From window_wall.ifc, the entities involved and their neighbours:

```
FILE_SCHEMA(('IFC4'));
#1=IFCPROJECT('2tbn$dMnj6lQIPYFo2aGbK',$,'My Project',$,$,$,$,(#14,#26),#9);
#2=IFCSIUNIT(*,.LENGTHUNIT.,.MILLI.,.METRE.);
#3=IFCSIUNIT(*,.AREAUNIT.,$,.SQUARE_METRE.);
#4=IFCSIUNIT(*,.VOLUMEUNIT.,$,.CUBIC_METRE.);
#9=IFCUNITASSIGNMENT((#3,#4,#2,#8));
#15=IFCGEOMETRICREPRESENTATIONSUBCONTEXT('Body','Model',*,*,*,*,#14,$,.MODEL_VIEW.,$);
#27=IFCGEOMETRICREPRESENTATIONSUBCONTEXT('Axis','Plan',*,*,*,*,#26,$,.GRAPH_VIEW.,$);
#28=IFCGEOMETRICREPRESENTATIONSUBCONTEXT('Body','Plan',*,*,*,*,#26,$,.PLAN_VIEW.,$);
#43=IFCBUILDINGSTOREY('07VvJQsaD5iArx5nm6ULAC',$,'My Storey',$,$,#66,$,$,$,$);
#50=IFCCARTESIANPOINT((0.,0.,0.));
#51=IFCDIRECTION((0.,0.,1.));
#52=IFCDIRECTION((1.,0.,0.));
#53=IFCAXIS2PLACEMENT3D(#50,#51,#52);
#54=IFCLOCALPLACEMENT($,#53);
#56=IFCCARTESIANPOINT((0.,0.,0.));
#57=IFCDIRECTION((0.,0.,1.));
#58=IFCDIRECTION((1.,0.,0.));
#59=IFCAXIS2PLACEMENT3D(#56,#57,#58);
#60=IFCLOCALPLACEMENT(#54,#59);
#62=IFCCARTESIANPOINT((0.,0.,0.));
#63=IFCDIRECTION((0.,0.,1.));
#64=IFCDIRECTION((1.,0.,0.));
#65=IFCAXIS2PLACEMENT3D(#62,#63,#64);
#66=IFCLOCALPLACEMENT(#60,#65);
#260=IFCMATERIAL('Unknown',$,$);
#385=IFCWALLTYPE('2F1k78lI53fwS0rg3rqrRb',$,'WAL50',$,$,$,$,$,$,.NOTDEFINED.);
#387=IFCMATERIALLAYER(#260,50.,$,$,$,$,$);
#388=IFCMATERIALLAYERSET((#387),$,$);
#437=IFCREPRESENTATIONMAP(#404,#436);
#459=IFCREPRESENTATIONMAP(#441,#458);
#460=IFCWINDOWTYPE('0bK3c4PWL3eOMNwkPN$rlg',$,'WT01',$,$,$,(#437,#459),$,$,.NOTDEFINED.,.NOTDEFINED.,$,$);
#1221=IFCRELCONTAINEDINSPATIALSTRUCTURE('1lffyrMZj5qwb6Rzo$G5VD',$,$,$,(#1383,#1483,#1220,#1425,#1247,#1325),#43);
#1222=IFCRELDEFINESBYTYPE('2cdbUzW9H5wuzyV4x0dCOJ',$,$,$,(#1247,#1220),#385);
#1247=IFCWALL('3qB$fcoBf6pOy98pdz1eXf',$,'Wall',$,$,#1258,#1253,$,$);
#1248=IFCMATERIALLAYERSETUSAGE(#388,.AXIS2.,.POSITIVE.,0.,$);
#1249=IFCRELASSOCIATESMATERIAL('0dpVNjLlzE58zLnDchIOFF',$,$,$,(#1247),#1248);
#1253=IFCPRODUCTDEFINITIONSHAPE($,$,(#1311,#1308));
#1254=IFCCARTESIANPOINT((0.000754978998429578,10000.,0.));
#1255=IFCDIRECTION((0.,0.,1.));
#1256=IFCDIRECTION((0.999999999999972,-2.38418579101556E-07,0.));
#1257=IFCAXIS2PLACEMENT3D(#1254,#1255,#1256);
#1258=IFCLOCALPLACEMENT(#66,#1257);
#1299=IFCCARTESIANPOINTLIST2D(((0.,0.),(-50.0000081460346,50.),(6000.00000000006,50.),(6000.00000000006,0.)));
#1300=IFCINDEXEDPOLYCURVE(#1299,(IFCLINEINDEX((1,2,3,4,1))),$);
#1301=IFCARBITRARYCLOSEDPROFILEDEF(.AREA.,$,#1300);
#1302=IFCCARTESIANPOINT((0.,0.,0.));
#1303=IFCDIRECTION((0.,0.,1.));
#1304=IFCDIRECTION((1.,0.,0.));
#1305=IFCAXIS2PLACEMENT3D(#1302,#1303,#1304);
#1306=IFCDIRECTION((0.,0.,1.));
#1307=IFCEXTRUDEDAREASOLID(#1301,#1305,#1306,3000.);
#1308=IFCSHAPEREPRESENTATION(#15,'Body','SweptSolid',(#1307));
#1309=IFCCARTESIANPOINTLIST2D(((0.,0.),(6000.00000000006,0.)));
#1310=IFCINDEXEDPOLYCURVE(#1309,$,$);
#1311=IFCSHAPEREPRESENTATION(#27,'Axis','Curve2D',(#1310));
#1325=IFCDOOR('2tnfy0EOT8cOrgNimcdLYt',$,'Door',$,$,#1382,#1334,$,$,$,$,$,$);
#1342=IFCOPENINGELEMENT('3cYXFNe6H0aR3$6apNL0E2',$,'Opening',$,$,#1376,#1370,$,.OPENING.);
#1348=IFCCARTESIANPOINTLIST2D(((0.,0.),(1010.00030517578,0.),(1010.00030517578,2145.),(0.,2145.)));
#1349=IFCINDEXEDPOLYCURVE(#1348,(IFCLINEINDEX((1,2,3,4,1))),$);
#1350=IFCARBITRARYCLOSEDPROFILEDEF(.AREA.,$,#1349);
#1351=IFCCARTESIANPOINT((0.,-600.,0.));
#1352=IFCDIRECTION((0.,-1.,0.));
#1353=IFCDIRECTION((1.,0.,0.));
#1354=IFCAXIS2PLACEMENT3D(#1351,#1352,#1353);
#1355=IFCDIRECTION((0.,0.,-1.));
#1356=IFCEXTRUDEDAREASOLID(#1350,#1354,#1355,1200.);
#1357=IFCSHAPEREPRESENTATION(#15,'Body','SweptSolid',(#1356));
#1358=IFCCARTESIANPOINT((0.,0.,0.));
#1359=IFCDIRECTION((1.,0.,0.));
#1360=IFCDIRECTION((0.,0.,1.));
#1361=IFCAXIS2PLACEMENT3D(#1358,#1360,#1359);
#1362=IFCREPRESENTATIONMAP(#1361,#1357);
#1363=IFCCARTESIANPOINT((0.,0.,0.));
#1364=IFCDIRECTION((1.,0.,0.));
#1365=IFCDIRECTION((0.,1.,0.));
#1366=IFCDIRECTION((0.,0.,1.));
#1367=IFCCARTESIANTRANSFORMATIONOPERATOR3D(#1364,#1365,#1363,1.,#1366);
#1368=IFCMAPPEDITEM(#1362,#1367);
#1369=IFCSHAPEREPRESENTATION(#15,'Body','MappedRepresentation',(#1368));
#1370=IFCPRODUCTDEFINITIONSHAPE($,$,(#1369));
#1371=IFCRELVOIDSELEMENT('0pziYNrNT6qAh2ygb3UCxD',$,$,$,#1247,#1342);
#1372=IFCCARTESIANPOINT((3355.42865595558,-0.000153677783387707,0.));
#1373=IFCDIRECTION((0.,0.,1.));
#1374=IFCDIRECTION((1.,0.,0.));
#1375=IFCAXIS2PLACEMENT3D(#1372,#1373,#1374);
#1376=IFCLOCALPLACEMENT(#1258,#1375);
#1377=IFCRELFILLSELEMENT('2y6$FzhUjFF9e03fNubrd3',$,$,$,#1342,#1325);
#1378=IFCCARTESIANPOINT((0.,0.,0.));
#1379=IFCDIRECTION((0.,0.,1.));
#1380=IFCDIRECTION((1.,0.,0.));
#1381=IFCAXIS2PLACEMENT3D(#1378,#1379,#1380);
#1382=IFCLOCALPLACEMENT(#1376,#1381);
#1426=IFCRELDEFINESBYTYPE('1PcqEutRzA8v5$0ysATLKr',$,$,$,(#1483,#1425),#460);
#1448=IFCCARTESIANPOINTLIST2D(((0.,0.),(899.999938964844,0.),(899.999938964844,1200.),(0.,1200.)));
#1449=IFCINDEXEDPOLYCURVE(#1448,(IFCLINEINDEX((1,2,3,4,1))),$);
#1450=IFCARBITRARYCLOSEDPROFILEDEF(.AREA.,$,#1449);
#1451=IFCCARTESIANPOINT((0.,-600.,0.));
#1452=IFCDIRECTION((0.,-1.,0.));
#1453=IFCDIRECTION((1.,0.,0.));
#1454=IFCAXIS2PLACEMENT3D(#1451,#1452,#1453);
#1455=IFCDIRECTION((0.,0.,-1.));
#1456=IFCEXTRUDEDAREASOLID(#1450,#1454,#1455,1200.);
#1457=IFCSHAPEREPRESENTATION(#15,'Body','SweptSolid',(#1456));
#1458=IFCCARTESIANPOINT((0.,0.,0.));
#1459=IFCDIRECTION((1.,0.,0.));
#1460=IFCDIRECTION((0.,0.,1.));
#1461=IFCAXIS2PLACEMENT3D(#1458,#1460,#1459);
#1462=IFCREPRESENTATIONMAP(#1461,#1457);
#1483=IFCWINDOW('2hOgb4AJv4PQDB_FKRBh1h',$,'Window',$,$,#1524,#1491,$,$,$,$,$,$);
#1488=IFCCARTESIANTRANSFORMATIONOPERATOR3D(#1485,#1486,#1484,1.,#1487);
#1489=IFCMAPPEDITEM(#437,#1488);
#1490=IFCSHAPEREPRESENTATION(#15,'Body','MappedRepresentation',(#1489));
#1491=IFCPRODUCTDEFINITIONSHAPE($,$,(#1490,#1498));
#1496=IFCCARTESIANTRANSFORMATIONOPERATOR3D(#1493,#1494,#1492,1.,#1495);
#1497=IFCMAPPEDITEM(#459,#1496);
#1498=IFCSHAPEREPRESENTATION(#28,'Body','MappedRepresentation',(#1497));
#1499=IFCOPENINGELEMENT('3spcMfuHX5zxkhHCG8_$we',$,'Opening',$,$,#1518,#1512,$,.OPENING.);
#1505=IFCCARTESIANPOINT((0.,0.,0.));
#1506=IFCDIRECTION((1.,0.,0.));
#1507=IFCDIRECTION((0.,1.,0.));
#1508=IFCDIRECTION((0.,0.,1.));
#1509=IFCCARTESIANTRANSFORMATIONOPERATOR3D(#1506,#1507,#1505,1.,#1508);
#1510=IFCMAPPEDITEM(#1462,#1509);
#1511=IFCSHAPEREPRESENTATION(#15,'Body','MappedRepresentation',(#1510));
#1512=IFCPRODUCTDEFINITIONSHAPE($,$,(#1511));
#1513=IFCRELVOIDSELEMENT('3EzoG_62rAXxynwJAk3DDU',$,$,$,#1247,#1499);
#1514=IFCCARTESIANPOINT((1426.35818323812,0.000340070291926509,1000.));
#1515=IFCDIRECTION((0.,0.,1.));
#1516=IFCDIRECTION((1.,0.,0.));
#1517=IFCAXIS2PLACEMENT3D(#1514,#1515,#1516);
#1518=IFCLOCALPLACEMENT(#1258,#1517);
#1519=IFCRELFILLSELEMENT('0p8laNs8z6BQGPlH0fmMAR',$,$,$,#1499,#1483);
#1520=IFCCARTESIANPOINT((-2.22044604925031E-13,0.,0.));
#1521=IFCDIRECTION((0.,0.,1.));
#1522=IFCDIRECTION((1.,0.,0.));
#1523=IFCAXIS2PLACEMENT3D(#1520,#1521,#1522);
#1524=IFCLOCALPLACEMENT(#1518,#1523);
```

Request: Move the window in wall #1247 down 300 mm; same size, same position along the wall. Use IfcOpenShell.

```python
import numpy as np
import ifcopenshell
import ifcopenshell.api.geometry
import ifcopenshell.util.placement
import ifcopenshell.util.unit

model = ifcopenshell.open("window_wall.ifc")
unit_scale = ifcopenshell.util.unit.calculate_unit_scale(model)

window = model.by_guid("2hOgb4AJv4PQDB_FKRBh1h")
opening = window.FillsVoids[0].RelatingOpeningElement
dz = -300.0

shift = np.array([0.0, 0.0, dz])
# The window is placed relative to its opening, so it follows when the opening moves.
matrix = ifcopenshell.util.placement.get_local_placement(opening.ObjectPlacement)
matrix[:3, 3] += shift
ifcopenshell.api.geometry.edit_object_placement(
    model, product=opening, matrix=matrix, is_si=False, should_transform_children=True
)

print(f"moved by {dz * unit_scale:+.3f} m")

model.write("window_wall-out.ifc")
```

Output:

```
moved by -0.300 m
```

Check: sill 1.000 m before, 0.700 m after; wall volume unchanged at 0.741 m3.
